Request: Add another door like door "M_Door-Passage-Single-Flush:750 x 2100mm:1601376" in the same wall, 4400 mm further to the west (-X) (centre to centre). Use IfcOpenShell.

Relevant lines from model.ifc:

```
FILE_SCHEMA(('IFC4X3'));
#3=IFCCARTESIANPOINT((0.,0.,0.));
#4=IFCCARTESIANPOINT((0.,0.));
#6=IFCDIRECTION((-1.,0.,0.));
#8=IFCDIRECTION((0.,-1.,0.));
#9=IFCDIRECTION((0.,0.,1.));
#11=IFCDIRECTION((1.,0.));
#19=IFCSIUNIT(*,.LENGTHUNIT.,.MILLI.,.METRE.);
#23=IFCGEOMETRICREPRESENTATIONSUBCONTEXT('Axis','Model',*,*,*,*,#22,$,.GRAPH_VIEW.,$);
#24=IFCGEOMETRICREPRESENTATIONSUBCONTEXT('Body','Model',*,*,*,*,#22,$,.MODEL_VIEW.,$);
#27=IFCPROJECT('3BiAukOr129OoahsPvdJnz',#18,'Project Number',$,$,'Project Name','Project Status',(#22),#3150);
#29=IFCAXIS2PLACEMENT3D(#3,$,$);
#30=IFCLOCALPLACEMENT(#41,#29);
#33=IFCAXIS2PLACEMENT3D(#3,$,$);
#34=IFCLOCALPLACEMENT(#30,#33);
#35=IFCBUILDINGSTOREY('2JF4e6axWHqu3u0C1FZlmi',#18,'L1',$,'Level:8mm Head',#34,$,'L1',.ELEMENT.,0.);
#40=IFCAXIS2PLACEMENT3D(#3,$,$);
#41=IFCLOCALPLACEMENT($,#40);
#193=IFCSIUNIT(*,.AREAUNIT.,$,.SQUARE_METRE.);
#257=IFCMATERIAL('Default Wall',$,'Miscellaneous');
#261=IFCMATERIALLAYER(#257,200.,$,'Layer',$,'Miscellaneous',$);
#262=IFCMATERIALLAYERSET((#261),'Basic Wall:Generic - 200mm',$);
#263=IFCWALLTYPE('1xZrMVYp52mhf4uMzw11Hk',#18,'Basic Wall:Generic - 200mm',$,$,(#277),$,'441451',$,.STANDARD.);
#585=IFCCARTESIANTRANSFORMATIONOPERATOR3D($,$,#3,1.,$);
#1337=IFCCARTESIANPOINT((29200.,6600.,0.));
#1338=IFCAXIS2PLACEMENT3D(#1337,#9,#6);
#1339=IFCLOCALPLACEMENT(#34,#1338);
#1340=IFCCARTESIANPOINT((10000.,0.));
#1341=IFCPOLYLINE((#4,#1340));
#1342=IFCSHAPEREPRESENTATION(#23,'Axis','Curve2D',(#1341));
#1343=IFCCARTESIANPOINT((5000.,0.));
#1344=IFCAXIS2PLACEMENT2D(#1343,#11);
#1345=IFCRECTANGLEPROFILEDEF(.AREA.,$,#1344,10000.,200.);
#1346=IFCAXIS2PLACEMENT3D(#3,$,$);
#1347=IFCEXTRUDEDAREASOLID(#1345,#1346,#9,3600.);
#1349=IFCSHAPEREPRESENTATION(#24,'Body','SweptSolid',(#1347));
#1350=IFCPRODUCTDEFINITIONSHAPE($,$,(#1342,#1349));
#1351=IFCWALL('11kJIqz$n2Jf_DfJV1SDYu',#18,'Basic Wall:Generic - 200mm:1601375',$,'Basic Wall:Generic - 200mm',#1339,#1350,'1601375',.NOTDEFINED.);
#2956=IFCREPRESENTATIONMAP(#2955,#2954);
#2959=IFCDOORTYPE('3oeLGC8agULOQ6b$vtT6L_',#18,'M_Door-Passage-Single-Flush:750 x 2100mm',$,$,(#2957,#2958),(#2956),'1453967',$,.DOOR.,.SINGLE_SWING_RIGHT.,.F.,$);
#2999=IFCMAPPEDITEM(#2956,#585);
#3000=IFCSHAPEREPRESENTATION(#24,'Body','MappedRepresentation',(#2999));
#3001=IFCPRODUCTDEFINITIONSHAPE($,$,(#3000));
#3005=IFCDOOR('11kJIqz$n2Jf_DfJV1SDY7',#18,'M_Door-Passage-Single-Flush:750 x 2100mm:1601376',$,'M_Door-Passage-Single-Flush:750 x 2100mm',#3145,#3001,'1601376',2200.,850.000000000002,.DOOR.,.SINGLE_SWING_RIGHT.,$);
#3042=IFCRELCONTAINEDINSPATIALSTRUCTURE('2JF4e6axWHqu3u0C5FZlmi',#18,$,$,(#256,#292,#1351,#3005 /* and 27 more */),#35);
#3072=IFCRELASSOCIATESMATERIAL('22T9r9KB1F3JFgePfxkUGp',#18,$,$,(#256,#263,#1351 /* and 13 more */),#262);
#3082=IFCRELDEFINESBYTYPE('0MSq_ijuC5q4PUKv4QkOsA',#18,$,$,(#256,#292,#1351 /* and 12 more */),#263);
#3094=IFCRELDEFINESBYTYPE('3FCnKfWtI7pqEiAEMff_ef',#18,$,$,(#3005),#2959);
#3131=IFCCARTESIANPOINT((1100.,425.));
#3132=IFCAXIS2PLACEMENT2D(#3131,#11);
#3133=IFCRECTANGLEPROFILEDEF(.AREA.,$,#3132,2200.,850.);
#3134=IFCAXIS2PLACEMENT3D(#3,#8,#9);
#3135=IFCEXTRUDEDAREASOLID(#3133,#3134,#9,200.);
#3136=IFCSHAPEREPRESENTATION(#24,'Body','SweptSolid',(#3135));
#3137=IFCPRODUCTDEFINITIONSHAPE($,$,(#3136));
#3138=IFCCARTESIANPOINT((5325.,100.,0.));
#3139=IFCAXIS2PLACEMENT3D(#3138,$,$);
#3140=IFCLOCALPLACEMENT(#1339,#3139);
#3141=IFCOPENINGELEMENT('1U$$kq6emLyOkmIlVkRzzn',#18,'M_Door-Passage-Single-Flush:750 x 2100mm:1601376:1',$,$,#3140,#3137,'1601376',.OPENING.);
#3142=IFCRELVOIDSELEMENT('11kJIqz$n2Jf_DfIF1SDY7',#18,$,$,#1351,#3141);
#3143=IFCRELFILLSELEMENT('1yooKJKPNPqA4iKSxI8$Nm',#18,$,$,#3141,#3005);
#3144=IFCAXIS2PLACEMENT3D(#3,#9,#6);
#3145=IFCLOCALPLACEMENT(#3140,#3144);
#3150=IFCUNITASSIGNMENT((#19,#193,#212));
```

```python
import ifcopenshell
import ifcopenshell.api.feature
import ifcopenshell.api.geometry
import ifcopenshell.api.root
import ifcopenshell.geom
import ifcopenshell.util.element
import ifcopenshell.util.placement
import ifcopenshell.util.shape
import ifcopenshell.util.unit

model = ifcopenshell.open("model.ifc")
unit_scale = ifcopenshell.util.unit.calculate_unit_scale(model)
settings = ifcopenshell.geom.settings()


def volume(element):
    """Net volume in cubic metres, openings subtracted."""
    shape = ifcopenshell.geom.create_shape(settings, element)
    return ifcopenshell.util.shape.get_volume(shape.geometry)


def reuse_history(source, copy):
    """copy_class also copies each property set's owner history, people and application; keep the originals."""
    for rel in copy.IsDefinedBy:
        if rel.is_a("IfcRelDefinesByProperties") and (history := rel.RelatingPropertyDefinition.OwnerHistory):
            rel.RelatingPropertyDefinition.OwnerHistory = source.OwnerHistory
            ifcopenshell.util.element.remove_deep2(model, history)


door = model.by_guid("11kJIqz$n2Jf_DfJV1SDY7")
opening = door.FillsVoids[0].RelatingOpeningElement
wall = opening.VoidsElements[0].RelatingBuildingElement
before = volume(wall)
shift = ifcopenshell.util.placement.get_local_placement(wall.ObjectPlacement)[:3, 0] * 4.4 / unit_scale

# copy_class copies the void relationship, type, container and properties, but no geometry.
new_opening = ifcopenshell.api.root.copy_class(model, product=opening)
new_opening.Representation = ifcopenshell.util.element.copy_deep(
    model, opening.Representation, exclude=["IfcGeometricRepresentationContext", "IfcRepresentationMap"]
)
new_opening.Name = "M_Door-Passage-Single-Flush:750 x 2100mm"
new_opening.Tag = None
new_door = ifcopenshell.api.root.copy_class(model, product=door)
new_door.Representation = ifcopenshell.util.element.copy_deep(
    model, door.Representation, exclude=["IfcGeometricRepresentationContext", "IfcRepresentationMap"]
)
new_door.Name = "M_Door-Passage-Single-Flush:750 x 2100mm"
new_door.Tag = None
reuse_history(door, new_door)
ifcopenshell.api.feature.add_filling(model, opening=new_opening, element=new_door)

for old, new in ((opening, new_opening), (door, new_door)):
    matrix = ifcopenshell.util.placement.get_local_placement(old.ObjectPlacement)
    matrix[:3, 3] += shift
    ifcopenshell.api.geometry.edit_object_placement(model, product=new, matrix=matrix, is_si=False)

after = volume(wall)

print(f"wall volume {before:.3f} -> {after:.3f} m3")

model.write("model_rev.ifc")
```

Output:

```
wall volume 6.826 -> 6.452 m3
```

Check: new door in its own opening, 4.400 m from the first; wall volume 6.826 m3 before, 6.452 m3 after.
